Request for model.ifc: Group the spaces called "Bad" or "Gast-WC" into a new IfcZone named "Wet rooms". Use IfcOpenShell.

First a look at what the model holds.

```python
import ifcopenshell

model = ifcopenshell.open("model.ifc")
print(model.schema)
seen = {}
for space in model.by_type("IfcSpace"):
    seen[space.LongName] = seen.get(space.LongName, 0) + 1
for name, count in sorted(seen.items(), key=str):
    print(count, "x", name)
print("zones:", [z.Name for z in model.by_type("IfcZone")][:20])
```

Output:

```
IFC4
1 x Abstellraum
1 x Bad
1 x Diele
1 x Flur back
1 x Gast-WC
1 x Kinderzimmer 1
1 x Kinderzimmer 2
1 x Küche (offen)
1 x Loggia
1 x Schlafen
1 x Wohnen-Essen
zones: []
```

```python
import ifcopenshell
import ifcopenshell.api.group
import ifcopenshell.api.root

model = ifcopenshell.open("model.ifc")

names = {"Bad", "Gast-WC"}
spaces = [s for s in model.by_type("IfcSpace") if s.LongName in names]

zone = ifcopenshell.api.root.create_entity(model, ifc_class="IfcZone", name="Wet rooms")
ifcopenshell.api.group.assign_group(model, products=spaces, group=zone)
print(len(spaces), "spaces in", zone.Name)

model.write("model_updated.ifc")
```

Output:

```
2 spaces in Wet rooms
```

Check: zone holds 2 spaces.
